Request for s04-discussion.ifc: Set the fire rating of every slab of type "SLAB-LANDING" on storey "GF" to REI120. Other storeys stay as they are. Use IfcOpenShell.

First a look at what the model holds.

```python
import ifcopenshell
import ifcopenshell.util.element

model = ifcopenshell.open("s04-discussion.ifc")
print(model.schema)
storey = next(s for s in model.by_type("IfcBuildingStorey") if s.Name == "GF")
slabs = [e for e in ifcopenshell.util.element.get_decomposition(storey) if e.is_a("IfcSlab")]
seen = {}
for e in slabs:
    element_type = ifcopenshell.util.element.get_type(e)
    key = (element_type.Name if element_type != e and element_type else None, ifcopenshell.util.element.get_pset(e, "Pset_SlabCommon", "FireRating"))
    seen[key] = seen.get(key, 0) + 1
for (name, value), count in sorted(seen.items(), key=str):
    print(count, "x", name, "|", value)
```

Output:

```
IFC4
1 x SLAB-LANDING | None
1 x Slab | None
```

```python
import ifcopenshell
import ifcopenshell.api.pset
import ifcopenshell.util.element

model = ifcopenshell.open("s04-discussion.ifc")

storey = next(s for s in model.by_type("IfcBuildingStorey") if s.Name == "GF")
slabs = [e for e in ifcopenshell.util.element.get_decomposition(storey) if e.is_a("IfcSlab")]

count = 0
for e in slabs:
    element_type = ifcopenshell.util.element.get_type(e)
    if element_type in (None, e) or element_type.Name != "SLAB-LANDING":
        continue
    # add_pset returns the element's existing set when there is one.
    pset = ifcopenshell.api.pset.add_pset(model, product=e, name="Pset_SlabCommon")
    ifcopenshell.api.pset.edit_pset(model, pset=pset, properties={"FireRating": "REI120"})
    count += 1

print(count, "slabs updated")

model.write("s04-discussion_rev.ifc")
```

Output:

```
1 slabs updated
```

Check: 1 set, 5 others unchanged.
